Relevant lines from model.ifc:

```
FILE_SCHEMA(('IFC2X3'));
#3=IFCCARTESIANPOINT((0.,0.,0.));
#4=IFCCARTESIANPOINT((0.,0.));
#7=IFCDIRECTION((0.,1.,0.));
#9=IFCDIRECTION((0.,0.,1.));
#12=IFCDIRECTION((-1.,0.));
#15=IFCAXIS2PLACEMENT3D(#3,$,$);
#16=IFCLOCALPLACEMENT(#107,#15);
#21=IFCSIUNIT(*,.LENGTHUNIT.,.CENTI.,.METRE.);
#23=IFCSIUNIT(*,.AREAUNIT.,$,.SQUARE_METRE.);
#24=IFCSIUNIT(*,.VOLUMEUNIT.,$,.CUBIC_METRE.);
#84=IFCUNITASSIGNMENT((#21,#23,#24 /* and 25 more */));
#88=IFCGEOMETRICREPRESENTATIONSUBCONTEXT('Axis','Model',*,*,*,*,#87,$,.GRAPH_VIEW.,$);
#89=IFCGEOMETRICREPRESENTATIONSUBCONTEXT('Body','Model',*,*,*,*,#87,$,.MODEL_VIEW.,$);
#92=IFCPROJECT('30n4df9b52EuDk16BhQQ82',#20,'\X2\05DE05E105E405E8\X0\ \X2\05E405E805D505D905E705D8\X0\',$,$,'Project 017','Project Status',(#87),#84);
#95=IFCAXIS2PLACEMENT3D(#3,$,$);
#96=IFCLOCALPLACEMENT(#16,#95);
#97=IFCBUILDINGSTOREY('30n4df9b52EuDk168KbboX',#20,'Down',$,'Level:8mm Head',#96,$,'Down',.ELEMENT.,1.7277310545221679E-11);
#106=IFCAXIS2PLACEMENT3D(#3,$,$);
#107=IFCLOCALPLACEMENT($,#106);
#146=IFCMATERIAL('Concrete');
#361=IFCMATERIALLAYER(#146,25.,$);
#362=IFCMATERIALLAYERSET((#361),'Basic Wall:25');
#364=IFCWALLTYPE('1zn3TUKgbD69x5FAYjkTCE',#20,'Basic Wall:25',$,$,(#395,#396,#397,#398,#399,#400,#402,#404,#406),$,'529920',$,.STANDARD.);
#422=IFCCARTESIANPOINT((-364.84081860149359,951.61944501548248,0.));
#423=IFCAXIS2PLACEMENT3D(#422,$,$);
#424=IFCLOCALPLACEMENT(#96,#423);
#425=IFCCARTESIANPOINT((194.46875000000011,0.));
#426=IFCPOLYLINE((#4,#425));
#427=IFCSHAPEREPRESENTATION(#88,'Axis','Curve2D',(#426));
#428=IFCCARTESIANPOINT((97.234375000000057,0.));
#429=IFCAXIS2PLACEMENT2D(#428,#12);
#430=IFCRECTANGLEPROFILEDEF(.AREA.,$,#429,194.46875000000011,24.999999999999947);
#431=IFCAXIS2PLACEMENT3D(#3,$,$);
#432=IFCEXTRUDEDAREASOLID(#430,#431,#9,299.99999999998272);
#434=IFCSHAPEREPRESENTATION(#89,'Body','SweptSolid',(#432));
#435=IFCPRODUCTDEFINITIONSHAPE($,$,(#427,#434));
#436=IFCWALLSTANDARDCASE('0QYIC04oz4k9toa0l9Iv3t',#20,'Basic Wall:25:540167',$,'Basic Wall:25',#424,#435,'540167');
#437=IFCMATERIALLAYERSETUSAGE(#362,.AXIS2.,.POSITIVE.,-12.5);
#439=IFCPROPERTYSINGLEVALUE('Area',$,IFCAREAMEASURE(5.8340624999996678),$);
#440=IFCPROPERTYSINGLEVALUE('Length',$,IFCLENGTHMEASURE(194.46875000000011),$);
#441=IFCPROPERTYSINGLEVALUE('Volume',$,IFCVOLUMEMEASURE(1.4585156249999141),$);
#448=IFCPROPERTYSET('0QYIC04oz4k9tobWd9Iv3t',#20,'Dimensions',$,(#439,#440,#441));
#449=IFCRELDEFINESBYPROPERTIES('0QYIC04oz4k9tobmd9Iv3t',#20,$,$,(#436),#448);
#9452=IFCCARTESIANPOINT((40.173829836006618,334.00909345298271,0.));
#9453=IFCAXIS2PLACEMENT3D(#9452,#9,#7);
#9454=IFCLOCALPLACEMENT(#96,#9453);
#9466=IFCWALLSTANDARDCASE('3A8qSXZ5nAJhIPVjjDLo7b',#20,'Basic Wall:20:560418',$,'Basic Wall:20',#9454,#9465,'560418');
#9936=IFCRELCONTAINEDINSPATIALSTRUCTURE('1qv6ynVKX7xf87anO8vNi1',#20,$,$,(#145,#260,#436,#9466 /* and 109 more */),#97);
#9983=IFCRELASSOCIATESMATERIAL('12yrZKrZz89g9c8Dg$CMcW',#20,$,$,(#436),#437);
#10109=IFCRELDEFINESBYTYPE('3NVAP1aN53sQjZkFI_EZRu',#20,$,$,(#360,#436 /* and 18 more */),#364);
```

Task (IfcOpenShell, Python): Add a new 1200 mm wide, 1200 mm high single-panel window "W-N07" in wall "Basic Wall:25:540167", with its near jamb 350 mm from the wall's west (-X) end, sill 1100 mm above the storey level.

```python
import numpy as np
import ifcopenshell
import ifcopenshell.api.feature
import ifcopenshell.api.geometry
import ifcopenshell.api.pset
import ifcopenshell.api.root
import ifcopenshell.api.spatial
import ifcopenshell.api.type
import ifcopenshell.geom
import ifcopenshell.util.element
import ifcopenshell.util.placement
import ifcopenshell.util.representation
import ifcopenshell.util.shape
import ifcopenshell.util.unit

model = ifcopenshell.open("model.ifc")
unit_scale = ifcopenshell.util.unit.calculate_unit_scale(model)
area_scale = ifcopenshell.util.unit.calculate_unit_scale(model, "AREAUNIT")
volume_scale = ifcopenshell.util.unit.calculate_unit_scale(model, "VOLUMEUNIT")
settings = ifcopenshell.geom.settings()


def volume(element):
    """Net volume in cubic metres, openings subtracted."""
    shape = ifcopenshell.geom.create_shape(settings, element)
    return ifcopenshell.util.shape.get_volume(shape.geometry)


wall = model.by_guid("0QYIC04oz4k9toa0l9Iv3t")
storey = ifcopenshell.util.element.get_container(wall, ifc_class="IfcBuildingStorey")
context = ifcopenshell.util.representation.get_context(model, "Model", "Body", "MODEL_VIEW")
before = volume(wall)

width, height, from_end, sill = 1.2, 1.2, 0.35, 1.1  # metres

# The wall runs along its own X axis, and the end named is its -X end.
wall_shape = ifcopenshell.geom.create_shape(settings, wall)
x, y, z = ifcopenshell.util.shape.get_vertices(wall_shape.geometry).T
start = x.min() + from_end
face, thickness = float(y.min()), float(y.max() - y.min())
wall_matrix = ifcopenshell.util.placement.get_local_placement(wall.ObjectPlacement)
level = ifcopenshell.util.placement.get_local_placement(storey.ObjectPlacement)[2, 3]


def in_wall(x, y):
    """Placement at x, y metres in the wall's axes, at sill height."""
    matrix = wall_matrix.copy()
    matrix[:, 3] = wall_matrix @ np.array([x / unit_scale, y / unit_scale, 0.0, 1.0])
    matrix[2, 3] = level + sill / unit_scale
    return matrix


# Opening: a box that overshoots both wall faces by 50 mm.
opening = ifcopenshell.api.root.create_entity(model, ifc_class="IfcOpeningElement")
box = ifcopenshell.api.geometry.add_wall_representation(
    model, context=context, length=width, height=height, thickness=thickness + 0.1
)
ifcopenshell.api.geometry.assign_representation(model, product=opening, representation=box)
ifcopenshell.api.geometry.edit_object_placement(model, product=opening, matrix=in_wall(start, face - 0.05), is_si=False)
ifcopenshell.api.feature.add_feature(model, feature=opening, element=wall)

window = ifcopenshell.api.root.create_entity(model, ifc_class="IfcWindow", name="W-N07")
window.OverallWidth, window.OverallHeight = width / unit_scale, height / unit_scale
body = ifcopenshell.api.geometry.add_window_representation(
    model,
    context=context,
    overall_width=window.OverallWidth,
    overall_height=window.OverallHeight,
    partition_type="SINGLE_PANEL",
)
ifcopenshell.api.geometry.assign_representation(model, product=window, representation=body)
ifcopenshell.api.spatial.assign_container(model, products=[window], relating_structure=storey)
fills = ifcopenshell.api.feature.add_filling(model, opening=opening, element=window)
fills.OwnerHistory = window.OwnerHistory  # required in IFC2X3

# IFC2X3 keeps the operation on the window style.
style = ifcopenshell.api.root.create_entity(model, ifc_class="IfcWindowStyle", name="W-N07")
style.OperationType, style.ConstructionType = "SINGLE_PANEL", "NOTDEFINED"
style.ParameterTakesPrecedence = style.Sizeable = False
ifcopenshell.api.type.assign_type(model, related_objects=[window], relating_type=style)

# Centre the window in the wall's thickness.
ifcopenshell.api.geometry.edit_object_placement(model, product=window, matrix=in_wall(start, face), is_si=False)
window_shape = ifcopenshell.geom.create_shape(settings, window)
depth = ifcopenshell.util.shape.get_vertices(window_shape.geometry)[:, 1]
offset = face + thickness / 2 - (depth.min() + depth.max()) / 2
ifcopenshell.api.geometry.edit_object_placement(model, product=window, matrix=in_wall(start, offset), is_si=False)

after = volume(wall)

# Update the wall's stored quantities.
pset = model.by_id(ifcopenshell.util.element.get_pset(wall, "Dimensions", should_inherit=False)["id"])
ifcopenshell.api.pset.edit_pset(model, pset=pset, properties={
    "Area": model.create_entity("IfcAreaMeasure", after / thickness / area_scale),
    "Volume": model.create_entity("IfcVolumeMeasure", after / volume_scale),
})

print(f"wall volume {before:.3f} -> {after:.3f} m3")

model.write("model_edited.ifc")
```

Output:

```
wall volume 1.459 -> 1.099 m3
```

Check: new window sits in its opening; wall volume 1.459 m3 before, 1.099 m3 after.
